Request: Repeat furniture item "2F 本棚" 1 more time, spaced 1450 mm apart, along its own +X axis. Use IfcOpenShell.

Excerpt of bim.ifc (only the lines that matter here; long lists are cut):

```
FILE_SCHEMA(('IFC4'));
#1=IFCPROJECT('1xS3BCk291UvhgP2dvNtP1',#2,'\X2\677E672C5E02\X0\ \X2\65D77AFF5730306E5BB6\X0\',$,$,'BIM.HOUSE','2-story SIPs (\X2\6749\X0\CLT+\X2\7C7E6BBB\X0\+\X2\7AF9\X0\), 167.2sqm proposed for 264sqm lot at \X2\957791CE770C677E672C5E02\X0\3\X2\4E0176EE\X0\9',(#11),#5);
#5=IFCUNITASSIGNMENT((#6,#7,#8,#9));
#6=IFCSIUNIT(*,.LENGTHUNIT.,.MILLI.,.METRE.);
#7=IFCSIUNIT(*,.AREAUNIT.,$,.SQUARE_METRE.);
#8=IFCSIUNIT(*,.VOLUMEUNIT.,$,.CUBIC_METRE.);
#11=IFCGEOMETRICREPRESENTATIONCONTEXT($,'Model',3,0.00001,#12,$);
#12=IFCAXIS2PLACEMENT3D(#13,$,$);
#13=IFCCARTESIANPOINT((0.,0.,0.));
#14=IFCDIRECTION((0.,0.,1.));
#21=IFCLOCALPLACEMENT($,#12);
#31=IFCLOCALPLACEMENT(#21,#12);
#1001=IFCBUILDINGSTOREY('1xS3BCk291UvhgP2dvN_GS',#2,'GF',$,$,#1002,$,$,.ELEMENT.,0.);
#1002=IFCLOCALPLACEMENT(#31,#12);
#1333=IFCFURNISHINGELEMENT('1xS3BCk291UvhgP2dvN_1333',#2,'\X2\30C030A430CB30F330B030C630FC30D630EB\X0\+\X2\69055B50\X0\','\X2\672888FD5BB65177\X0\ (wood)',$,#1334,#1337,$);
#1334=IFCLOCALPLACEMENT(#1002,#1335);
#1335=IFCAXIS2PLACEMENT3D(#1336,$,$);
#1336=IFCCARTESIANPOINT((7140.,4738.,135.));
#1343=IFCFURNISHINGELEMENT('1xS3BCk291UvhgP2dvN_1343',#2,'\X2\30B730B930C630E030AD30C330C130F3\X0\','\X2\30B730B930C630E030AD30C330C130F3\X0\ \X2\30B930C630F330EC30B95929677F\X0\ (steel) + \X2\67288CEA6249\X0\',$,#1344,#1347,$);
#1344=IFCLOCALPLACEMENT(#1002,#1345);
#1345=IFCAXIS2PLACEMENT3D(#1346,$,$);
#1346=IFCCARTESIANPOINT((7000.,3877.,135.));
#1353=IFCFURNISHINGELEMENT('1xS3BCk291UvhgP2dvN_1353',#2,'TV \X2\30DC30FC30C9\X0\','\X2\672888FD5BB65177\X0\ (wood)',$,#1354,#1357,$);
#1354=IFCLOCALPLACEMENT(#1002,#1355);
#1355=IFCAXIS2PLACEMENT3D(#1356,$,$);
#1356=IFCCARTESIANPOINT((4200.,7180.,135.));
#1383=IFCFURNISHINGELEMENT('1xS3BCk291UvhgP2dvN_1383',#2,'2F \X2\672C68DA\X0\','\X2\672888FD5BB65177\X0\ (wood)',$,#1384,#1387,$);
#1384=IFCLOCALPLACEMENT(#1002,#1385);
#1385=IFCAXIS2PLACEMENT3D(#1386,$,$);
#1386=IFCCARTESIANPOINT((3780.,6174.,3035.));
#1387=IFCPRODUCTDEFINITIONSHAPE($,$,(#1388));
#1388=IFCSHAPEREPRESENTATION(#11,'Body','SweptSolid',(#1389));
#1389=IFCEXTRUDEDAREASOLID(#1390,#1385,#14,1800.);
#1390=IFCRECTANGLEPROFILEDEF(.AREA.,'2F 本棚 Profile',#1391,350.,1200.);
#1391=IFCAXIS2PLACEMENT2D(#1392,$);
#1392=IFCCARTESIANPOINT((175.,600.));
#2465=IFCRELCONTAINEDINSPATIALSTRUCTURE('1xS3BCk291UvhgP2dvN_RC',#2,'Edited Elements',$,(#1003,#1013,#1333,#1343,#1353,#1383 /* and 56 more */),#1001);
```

```python
import ifcopenshell
import ifcopenshell.api.geometry
import ifcopenshell.api.root
import ifcopenshell.util.element
import ifcopenshell.util.placement
import ifcopenshell.util.unit

model = ifcopenshell.open("bim.ifc")
unit_scale = ifcopenshell.util.unit.calculate_unit_scale(model)


def reuse_history(source, copy):
    """copy_class also copies each property set's owner history, people and application; keep the originals."""
    for rel in copy.IsDefinedBy:
        if rel.is_a("IfcRelDefinesByProperties") and (history := rel.RelatingPropertyDefinition.OwnerHistory):
            rel.RelatingPropertyDefinition.OwnerHistory = source.OwnerHistory
            ifcopenshell.util.element.remove_deep2(model, history)


source = model.by_guid("1xS3BCk291UvhgP2dvN_1383")
base = ifcopenshell.util.placement.get_local_placement(source.ObjectPlacement)
step = base[:3, 0] * 1.45 / unit_scale

for i in range(1, 2):
    copy = ifcopenshell.api.root.copy_class(model, product=source)
    copy.Representation = ifcopenshell.util.element.copy_deep(
        model, source.Representation, exclude=["IfcGeometricRepresentationContext", "IfcRepresentationMap"]
    )
    reuse_history(source, copy)
    matrix = base.copy()
    matrix[:3, 3] += i * step
    print("added at", matrix[:3, 3].round(3) + 0.0)
    ifcopenshell.api.geometry.edit_object_placement(model, product=copy, matrix=matrix, is_si=False)

model.write("bim_v2.ifc")
```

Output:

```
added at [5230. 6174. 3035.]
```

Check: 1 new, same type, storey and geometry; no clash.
